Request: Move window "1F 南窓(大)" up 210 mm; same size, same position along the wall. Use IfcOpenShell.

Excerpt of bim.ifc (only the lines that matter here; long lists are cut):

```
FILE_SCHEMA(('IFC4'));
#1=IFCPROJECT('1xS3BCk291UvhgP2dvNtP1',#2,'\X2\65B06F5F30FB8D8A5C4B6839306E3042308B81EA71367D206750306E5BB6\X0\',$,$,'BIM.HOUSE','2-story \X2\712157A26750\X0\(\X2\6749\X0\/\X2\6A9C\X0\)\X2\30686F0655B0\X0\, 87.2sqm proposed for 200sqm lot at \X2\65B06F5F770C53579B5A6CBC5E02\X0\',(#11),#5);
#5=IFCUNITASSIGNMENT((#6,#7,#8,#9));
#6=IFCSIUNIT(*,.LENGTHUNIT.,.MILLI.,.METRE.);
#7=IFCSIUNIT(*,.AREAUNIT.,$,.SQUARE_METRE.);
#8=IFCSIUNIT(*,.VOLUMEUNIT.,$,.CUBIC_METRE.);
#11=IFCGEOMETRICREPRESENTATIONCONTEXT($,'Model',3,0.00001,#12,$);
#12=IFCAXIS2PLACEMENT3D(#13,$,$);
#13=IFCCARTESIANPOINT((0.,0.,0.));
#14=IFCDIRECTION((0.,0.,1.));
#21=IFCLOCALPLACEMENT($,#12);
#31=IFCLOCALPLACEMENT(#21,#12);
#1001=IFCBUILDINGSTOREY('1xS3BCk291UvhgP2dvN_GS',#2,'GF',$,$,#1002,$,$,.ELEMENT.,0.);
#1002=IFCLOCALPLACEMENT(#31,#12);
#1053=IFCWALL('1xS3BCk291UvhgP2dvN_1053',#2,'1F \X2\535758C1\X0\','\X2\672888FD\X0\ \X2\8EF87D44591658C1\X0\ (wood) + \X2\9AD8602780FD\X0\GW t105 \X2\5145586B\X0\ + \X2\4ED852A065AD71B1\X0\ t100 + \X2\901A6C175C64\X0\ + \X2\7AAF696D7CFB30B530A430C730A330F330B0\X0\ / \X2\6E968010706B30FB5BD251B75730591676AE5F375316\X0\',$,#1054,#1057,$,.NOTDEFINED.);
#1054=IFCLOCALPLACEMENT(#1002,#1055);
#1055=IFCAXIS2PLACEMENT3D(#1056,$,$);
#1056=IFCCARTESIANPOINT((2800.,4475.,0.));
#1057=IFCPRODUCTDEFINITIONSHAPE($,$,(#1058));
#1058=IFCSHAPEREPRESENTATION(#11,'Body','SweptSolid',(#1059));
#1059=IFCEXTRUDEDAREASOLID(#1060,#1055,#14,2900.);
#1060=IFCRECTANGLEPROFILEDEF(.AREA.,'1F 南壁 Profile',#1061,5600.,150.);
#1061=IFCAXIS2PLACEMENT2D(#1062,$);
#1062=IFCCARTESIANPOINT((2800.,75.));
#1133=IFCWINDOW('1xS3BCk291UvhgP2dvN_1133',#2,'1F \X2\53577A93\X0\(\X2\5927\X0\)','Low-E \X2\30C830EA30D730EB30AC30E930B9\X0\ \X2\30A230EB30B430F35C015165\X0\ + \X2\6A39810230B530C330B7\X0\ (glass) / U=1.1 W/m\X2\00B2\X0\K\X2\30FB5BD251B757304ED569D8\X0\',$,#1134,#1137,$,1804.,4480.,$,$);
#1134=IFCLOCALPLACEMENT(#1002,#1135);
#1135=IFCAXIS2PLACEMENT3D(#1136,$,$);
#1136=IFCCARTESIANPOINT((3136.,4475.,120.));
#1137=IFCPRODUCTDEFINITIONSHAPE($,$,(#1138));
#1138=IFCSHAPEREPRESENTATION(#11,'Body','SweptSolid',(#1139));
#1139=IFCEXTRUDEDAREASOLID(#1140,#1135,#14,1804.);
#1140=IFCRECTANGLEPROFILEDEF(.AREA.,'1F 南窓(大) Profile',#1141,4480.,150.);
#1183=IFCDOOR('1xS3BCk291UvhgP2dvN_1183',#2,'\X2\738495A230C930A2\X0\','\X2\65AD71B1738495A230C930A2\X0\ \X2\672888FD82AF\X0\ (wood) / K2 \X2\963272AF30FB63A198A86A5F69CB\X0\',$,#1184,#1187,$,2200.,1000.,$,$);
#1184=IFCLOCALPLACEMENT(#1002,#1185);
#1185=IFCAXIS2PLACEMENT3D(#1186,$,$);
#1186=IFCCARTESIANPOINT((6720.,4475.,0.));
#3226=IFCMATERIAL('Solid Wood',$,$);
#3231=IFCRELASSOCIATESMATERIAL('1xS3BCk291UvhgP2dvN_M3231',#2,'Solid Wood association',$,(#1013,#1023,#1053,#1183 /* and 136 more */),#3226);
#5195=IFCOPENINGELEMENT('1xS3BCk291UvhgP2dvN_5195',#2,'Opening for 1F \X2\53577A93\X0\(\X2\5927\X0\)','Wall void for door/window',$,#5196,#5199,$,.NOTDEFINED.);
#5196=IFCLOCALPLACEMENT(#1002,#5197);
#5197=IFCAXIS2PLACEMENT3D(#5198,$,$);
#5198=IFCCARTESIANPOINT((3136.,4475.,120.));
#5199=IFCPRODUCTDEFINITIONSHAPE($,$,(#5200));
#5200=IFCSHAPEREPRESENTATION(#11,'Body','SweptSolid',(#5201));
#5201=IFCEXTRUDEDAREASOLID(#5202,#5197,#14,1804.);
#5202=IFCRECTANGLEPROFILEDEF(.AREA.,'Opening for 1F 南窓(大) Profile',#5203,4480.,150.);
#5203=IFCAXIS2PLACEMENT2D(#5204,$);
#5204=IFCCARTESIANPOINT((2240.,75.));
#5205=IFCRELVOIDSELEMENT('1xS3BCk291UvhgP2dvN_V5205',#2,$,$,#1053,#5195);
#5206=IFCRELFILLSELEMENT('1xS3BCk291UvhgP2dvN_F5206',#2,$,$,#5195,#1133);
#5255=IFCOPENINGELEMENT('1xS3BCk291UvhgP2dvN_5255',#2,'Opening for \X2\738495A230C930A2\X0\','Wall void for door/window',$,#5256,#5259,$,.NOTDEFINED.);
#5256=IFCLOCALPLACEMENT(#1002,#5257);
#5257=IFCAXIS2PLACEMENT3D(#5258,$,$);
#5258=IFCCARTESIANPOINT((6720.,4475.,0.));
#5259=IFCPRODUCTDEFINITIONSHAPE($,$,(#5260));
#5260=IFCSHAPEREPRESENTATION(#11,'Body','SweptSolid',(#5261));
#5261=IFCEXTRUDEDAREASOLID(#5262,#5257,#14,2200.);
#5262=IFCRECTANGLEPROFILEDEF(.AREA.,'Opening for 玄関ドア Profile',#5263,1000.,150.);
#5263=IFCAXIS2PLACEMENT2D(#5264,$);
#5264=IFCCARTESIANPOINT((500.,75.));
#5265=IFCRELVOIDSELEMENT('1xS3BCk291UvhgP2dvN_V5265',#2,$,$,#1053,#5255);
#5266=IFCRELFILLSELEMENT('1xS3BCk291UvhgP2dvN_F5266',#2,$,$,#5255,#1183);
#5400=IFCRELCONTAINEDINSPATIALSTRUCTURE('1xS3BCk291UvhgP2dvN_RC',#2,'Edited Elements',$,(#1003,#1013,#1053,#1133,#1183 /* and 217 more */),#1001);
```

```python
import numpy as np
import ifcopenshell
import ifcopenshell.api.geometry
import ifcopenshell.util.placement
import ifcopenshell.util.unit

model = ifcopenshell.open("bim.ifc")
unit_scale = ifcopenshell.util.unit.calculate_unit_scale(model)

window = model.by_id(1133)
opening = window.FillsVoids[0].RelatingOpeningElement
dz = 210.0

shift = np.array([0.0, 0.0, dz])
# The window is not placed relative to its opening, so move both.
for product in (opening, window):
    matrix = ifcopenshell.util.placement.get_local_placement(product.ObjectPlacement)
    matrix[:3, 3] += shift
    ifcopenshell.api.geometry.edit_object_placement(model, product=product, matrix=matrix, is_si=False)

print(f"moved by {dz * unit_scale:+.3f} m")

model.write("bim_rev.ifc")
```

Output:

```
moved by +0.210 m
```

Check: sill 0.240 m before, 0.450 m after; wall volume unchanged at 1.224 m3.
